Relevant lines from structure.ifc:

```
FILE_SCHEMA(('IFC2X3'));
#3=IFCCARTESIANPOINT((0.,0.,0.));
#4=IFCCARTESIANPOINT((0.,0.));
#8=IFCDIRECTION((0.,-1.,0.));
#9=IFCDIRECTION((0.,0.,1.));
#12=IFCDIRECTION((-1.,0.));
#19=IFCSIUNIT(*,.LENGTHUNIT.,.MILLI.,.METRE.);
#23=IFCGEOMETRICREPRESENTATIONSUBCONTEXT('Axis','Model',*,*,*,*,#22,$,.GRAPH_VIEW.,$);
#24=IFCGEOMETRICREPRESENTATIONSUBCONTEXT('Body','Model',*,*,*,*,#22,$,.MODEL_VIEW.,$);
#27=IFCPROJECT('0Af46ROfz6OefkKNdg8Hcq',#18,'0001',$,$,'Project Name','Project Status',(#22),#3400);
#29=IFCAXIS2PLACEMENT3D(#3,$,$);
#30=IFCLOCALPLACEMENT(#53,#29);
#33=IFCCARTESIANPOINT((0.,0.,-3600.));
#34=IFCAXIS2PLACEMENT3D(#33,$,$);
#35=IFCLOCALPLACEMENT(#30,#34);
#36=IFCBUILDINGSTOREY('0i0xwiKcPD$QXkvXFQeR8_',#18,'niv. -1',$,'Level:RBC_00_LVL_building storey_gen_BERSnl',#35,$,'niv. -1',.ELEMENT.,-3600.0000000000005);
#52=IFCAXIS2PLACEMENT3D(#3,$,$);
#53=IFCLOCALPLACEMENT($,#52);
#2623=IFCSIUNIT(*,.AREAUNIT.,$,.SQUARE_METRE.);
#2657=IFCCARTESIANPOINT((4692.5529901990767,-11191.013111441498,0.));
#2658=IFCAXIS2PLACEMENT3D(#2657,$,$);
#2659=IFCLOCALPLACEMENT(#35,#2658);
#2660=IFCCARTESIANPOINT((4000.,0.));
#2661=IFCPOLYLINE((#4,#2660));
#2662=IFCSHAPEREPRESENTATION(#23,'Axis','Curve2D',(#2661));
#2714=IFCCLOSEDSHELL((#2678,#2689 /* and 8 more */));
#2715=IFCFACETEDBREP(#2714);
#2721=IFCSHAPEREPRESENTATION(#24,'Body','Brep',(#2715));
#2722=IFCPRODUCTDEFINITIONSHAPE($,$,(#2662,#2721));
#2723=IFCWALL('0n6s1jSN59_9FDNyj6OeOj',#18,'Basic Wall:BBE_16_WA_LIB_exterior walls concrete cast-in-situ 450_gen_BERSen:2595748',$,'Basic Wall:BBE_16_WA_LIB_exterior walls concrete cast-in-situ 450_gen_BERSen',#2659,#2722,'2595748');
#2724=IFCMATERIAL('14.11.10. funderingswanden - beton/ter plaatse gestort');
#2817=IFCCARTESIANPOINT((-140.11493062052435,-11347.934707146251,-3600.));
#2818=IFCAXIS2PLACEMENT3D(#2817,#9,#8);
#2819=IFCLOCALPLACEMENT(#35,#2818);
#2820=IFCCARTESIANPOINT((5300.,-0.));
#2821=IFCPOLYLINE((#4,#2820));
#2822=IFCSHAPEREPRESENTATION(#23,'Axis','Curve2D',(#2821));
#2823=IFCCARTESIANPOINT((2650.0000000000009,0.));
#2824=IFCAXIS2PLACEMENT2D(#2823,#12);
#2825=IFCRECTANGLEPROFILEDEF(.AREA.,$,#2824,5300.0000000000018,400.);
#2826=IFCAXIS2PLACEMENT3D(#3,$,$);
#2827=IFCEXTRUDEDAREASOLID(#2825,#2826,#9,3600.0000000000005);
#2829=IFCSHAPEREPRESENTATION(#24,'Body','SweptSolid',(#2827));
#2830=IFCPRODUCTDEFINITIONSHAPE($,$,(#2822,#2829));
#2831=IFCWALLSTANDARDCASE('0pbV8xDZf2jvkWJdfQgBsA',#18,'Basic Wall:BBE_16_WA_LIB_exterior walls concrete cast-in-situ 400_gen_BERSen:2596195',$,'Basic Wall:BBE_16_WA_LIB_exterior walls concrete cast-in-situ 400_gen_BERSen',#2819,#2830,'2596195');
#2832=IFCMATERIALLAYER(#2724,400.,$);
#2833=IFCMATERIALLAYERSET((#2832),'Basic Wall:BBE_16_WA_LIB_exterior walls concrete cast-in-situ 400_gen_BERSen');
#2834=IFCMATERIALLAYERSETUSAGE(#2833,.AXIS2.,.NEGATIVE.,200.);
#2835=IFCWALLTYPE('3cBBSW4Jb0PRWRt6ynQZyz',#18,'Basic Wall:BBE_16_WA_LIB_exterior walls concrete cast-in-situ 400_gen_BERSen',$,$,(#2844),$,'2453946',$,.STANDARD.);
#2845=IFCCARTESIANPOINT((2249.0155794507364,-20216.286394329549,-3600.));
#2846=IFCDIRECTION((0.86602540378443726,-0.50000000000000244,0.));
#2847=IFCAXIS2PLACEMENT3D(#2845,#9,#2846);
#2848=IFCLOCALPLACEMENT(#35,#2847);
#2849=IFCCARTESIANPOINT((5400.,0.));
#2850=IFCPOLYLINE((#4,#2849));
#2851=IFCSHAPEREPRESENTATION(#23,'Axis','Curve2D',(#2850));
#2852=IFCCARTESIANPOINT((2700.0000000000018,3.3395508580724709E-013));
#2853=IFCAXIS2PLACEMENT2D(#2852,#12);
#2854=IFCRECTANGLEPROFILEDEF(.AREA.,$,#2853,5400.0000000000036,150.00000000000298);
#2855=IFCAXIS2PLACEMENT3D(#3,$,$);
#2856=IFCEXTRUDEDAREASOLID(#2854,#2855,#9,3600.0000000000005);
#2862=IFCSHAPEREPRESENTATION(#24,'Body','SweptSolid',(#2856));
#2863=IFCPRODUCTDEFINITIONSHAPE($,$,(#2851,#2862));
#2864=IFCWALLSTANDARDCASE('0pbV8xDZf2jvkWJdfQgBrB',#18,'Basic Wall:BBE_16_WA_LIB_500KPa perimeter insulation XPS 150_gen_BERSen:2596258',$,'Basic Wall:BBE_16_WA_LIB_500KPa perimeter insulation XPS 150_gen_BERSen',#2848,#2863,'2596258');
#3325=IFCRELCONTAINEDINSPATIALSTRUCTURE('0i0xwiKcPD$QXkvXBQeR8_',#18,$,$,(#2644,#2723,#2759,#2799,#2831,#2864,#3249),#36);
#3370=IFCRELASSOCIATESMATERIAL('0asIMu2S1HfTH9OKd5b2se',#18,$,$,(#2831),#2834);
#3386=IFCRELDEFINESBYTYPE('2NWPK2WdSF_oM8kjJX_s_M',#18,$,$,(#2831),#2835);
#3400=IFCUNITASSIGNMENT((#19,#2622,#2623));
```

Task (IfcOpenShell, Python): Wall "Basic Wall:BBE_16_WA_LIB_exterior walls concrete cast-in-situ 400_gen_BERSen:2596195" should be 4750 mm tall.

```python
import ifcopenshell
import ifcopenshell.geom
import ifcopenshell.util.representation
import ifcopenshell.util.shape
import ifcopenshell.util.unit

model = ifcopenshell.open("structure.ifc")
unit_scale = ifcopenshell.util.unit.calculate_unit_scale(model)
settings = ifcopenshell.geom.settings()


def volume(element):
    """Net volume in cubic metres, openings subtracted."""
    shape = ifcopenshell.geom.create_shape(settings, element)
    return ifcopenshell.util.shape.get_volume(shape.geometry)


wall = model.by_id(2831)
before = volume(wall)

body = ifcopenshell.util.representation.get_representation(wall, "Model", "Body")
solid = body.Items[0]
old_height = solid.Depth
solid.Depth = 4.75 / unit_scale
after = volume(wall)

print(f"height {old_height:g} -> {solid.Depth:g}, volume {before:.3f} -> {after:.3f} m3")

model.write("structure-out.ifc")
```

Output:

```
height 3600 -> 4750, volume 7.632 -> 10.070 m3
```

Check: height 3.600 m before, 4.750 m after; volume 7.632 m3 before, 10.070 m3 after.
